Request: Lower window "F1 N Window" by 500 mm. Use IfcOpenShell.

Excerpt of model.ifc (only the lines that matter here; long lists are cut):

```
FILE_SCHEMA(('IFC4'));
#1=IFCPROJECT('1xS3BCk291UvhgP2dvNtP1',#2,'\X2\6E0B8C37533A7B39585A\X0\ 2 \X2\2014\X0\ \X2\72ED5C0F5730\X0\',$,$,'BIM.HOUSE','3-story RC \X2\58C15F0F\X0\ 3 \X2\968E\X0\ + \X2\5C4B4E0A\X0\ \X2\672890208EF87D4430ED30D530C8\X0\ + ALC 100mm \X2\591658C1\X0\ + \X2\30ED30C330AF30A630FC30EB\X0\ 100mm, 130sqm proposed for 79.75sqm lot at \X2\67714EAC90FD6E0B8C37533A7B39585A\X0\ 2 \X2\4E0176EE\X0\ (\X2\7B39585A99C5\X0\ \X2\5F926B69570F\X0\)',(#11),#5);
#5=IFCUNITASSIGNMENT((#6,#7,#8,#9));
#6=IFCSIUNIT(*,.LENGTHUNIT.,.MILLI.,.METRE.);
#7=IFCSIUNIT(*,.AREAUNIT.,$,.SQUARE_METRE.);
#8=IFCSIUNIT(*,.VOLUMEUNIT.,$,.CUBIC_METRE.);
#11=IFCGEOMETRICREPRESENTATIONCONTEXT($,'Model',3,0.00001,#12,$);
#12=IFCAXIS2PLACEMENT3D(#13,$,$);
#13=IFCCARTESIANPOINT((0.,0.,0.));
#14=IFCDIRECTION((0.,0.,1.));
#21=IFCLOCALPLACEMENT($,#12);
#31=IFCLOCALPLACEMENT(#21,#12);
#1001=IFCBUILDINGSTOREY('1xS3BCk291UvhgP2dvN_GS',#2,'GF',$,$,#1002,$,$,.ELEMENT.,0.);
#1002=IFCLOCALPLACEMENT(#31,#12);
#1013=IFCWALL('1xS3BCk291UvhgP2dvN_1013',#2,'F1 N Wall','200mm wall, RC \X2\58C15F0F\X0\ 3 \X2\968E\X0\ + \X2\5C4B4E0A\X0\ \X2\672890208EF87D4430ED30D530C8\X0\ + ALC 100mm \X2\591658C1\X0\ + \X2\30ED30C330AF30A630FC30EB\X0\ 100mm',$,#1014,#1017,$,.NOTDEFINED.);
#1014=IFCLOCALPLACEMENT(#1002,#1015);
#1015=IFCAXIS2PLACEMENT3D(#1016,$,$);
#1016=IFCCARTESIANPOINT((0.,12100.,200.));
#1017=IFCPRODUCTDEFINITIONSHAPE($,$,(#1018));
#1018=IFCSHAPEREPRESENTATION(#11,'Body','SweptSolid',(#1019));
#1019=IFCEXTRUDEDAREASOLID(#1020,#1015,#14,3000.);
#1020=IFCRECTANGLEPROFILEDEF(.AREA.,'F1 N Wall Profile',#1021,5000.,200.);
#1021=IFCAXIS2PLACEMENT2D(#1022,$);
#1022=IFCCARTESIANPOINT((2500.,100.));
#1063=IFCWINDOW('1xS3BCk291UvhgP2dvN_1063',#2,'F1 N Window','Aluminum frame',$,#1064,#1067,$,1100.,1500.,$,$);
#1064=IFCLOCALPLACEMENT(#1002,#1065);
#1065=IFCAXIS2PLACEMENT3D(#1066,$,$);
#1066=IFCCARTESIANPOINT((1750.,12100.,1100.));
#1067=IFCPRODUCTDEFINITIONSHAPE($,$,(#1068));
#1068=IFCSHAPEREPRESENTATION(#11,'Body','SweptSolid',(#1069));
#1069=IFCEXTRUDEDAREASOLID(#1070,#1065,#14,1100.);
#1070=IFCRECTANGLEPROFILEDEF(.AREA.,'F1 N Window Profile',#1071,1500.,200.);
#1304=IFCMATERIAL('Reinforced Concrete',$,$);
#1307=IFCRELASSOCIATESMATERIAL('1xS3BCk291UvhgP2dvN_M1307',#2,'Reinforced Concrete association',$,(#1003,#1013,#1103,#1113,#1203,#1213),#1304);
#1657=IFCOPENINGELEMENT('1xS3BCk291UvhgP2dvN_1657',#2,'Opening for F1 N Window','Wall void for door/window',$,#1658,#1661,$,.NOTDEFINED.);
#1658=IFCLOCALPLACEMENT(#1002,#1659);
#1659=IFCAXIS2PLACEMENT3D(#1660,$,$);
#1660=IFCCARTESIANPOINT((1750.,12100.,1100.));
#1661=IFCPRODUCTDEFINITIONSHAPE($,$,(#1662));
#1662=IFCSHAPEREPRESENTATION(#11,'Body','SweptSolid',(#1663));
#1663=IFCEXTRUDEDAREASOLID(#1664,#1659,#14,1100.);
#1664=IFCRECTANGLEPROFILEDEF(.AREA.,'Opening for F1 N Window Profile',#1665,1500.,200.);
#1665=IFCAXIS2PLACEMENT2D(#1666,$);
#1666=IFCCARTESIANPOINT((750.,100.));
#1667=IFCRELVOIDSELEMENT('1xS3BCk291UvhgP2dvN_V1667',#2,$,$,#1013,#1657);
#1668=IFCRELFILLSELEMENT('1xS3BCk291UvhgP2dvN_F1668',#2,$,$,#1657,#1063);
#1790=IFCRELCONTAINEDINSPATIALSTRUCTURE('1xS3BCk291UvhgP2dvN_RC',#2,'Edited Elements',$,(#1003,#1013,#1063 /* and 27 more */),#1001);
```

```python
import numpy as np
import ifcopenshell
import ifcopenshell.api.geometry
import ifcopenshell.util.placement
import ifcopenshell.util.unit

model = ifcopenshell.open("model.ifc")
unit_scale = ifcopenshell.util.unit.calculate_unit_scale(model)

window = model.by_guid("1xS3BCk291UvhgP2dvN_1063")
opening = window.FillsVoids[0].RelatingOpeningElement
dz = -500.0

shift = np.array([0.0, 0.0, dz])
# The window is not placed relative to its opening, so move both.
for product in (opening, window):
    matrix = ifcopenshell.util.placement.get_local_placement(product.ObjectPlacement)
    matrix[:3, 3] += shift
    ifcopenshell.api.geometry.edit_object_placement(model, product=product, matrix=matrix, is_si=False)

print(f"moved by {dz * unit_scale:+.3f} m")

model.write("model_edited.ifc")
```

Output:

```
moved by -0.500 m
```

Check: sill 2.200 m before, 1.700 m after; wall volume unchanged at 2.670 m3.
